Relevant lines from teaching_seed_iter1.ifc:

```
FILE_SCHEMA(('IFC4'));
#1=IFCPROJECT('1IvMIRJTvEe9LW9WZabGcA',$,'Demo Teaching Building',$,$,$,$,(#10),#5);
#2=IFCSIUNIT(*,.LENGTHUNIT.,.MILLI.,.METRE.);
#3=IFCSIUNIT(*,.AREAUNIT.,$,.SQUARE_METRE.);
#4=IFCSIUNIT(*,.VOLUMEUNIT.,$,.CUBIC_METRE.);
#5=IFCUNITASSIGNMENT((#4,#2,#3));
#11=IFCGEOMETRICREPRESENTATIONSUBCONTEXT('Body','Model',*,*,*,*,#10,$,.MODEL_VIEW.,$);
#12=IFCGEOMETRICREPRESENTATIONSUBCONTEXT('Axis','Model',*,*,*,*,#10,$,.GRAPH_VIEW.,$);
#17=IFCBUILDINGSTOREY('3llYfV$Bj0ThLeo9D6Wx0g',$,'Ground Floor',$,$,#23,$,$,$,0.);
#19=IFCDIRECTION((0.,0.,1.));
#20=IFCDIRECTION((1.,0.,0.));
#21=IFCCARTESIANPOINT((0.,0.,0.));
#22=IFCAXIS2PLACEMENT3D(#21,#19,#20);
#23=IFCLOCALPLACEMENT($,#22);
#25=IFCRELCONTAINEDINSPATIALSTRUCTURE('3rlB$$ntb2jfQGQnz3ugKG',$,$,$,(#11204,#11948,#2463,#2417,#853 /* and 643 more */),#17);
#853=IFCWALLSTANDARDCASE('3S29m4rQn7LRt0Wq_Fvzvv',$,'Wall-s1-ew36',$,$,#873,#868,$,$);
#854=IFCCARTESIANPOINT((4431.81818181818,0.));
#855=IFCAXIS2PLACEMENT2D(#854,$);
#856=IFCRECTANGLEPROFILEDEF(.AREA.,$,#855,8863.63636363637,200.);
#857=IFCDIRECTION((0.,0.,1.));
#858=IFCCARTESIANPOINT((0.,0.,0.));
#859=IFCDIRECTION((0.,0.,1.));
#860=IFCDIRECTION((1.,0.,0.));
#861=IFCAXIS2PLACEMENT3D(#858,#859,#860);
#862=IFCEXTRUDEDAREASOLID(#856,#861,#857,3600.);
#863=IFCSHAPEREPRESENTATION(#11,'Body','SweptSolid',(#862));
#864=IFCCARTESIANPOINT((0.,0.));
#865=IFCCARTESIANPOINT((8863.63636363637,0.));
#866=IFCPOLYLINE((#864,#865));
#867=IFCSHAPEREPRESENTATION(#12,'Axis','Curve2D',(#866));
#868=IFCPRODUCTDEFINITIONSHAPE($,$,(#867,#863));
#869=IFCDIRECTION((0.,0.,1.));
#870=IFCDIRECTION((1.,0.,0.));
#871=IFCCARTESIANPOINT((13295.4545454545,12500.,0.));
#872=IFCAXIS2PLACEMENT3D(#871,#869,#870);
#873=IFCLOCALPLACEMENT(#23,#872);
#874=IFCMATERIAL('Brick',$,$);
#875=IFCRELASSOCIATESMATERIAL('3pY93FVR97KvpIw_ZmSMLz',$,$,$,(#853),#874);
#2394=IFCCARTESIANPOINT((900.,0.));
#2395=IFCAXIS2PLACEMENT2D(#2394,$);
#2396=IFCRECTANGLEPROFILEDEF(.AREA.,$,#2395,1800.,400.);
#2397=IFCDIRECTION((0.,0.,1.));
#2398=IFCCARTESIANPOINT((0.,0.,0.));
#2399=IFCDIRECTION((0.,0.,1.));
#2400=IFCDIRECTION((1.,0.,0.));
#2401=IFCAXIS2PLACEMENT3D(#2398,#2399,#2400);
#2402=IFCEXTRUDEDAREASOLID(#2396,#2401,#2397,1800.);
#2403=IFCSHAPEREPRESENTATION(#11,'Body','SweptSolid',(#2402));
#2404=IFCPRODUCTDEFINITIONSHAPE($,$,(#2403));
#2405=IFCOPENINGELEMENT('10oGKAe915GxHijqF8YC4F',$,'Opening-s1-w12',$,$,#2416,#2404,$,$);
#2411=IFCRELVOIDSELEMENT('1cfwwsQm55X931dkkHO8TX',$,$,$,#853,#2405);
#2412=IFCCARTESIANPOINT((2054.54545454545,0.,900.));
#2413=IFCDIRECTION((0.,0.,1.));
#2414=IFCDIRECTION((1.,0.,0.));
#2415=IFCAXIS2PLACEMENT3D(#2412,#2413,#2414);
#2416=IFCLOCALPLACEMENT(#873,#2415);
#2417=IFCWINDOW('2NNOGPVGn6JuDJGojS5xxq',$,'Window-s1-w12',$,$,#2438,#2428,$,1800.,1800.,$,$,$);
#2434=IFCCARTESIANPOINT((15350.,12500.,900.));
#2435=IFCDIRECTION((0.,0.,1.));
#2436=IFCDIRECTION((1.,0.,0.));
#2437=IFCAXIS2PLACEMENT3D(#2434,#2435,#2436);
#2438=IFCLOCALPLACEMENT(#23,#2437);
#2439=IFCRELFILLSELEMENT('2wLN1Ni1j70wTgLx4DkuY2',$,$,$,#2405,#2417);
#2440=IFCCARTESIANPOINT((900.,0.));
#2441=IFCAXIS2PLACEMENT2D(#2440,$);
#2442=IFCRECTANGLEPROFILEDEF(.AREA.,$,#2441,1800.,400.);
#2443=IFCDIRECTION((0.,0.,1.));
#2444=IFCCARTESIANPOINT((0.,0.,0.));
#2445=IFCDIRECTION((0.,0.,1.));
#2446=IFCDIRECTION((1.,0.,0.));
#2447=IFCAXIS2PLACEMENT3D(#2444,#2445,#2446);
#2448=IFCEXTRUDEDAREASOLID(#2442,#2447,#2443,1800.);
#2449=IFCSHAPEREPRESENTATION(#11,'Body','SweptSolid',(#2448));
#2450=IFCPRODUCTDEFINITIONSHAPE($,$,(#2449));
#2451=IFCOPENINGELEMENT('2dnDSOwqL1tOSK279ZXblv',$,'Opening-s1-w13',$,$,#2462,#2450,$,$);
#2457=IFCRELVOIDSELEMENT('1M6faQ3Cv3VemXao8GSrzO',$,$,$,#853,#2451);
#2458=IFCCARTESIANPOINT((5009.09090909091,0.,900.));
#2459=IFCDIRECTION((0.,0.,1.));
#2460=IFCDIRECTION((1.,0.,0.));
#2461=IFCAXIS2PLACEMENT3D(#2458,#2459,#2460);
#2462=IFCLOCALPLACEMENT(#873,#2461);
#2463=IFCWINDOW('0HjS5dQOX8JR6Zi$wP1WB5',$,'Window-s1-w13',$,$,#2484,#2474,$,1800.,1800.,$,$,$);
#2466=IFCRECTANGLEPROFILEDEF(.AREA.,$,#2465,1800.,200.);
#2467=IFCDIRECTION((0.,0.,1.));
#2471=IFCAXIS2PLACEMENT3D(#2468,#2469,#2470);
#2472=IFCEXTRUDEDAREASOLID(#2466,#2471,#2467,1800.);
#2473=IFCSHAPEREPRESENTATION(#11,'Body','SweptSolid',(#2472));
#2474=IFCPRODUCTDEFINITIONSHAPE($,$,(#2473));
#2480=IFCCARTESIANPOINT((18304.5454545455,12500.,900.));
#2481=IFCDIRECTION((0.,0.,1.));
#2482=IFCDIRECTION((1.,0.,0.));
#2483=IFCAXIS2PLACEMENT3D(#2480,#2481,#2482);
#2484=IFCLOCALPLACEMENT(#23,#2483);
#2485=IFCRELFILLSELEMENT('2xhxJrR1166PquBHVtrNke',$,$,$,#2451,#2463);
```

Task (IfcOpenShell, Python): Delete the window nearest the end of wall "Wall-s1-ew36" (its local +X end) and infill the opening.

```python
import ifcopenshell
import ifcopenshell.api.feature
import ifcopenshell.api.root
import ifcopenshell.geom
import ifcopenshell.util.shape

model = ifcopenshell.open("teaching_seed_iter1.ifc")
settings = ifcopenshell.geom.settings()


def volume(element):
    """Net volume in cubic metres, openings subtracted."""
    shape = ifcopenshell.geom.create_shape(settings, element)
    return ifcopenshell.util.shape.get_volume(shape.geometry)


window = model.by_id(2463)
opening = window.FillsVoids[0].RelatingOpeningElement
wall = opening.VoidsElements[0].RelatingBuildingElement
before = volume(wall)

ifcopenshell.api.root.remove_product(model, product=window)
ifcopenshell.api.feature.remove_feature(model, feature=opening)

after = volume(wall)

print(f"wall volume {before:.3f} -> {after:.3f} m3")

model.write("teaching_seed_iter1_rev.ifc")
```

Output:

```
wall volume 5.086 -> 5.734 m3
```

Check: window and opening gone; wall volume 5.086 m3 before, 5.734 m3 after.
